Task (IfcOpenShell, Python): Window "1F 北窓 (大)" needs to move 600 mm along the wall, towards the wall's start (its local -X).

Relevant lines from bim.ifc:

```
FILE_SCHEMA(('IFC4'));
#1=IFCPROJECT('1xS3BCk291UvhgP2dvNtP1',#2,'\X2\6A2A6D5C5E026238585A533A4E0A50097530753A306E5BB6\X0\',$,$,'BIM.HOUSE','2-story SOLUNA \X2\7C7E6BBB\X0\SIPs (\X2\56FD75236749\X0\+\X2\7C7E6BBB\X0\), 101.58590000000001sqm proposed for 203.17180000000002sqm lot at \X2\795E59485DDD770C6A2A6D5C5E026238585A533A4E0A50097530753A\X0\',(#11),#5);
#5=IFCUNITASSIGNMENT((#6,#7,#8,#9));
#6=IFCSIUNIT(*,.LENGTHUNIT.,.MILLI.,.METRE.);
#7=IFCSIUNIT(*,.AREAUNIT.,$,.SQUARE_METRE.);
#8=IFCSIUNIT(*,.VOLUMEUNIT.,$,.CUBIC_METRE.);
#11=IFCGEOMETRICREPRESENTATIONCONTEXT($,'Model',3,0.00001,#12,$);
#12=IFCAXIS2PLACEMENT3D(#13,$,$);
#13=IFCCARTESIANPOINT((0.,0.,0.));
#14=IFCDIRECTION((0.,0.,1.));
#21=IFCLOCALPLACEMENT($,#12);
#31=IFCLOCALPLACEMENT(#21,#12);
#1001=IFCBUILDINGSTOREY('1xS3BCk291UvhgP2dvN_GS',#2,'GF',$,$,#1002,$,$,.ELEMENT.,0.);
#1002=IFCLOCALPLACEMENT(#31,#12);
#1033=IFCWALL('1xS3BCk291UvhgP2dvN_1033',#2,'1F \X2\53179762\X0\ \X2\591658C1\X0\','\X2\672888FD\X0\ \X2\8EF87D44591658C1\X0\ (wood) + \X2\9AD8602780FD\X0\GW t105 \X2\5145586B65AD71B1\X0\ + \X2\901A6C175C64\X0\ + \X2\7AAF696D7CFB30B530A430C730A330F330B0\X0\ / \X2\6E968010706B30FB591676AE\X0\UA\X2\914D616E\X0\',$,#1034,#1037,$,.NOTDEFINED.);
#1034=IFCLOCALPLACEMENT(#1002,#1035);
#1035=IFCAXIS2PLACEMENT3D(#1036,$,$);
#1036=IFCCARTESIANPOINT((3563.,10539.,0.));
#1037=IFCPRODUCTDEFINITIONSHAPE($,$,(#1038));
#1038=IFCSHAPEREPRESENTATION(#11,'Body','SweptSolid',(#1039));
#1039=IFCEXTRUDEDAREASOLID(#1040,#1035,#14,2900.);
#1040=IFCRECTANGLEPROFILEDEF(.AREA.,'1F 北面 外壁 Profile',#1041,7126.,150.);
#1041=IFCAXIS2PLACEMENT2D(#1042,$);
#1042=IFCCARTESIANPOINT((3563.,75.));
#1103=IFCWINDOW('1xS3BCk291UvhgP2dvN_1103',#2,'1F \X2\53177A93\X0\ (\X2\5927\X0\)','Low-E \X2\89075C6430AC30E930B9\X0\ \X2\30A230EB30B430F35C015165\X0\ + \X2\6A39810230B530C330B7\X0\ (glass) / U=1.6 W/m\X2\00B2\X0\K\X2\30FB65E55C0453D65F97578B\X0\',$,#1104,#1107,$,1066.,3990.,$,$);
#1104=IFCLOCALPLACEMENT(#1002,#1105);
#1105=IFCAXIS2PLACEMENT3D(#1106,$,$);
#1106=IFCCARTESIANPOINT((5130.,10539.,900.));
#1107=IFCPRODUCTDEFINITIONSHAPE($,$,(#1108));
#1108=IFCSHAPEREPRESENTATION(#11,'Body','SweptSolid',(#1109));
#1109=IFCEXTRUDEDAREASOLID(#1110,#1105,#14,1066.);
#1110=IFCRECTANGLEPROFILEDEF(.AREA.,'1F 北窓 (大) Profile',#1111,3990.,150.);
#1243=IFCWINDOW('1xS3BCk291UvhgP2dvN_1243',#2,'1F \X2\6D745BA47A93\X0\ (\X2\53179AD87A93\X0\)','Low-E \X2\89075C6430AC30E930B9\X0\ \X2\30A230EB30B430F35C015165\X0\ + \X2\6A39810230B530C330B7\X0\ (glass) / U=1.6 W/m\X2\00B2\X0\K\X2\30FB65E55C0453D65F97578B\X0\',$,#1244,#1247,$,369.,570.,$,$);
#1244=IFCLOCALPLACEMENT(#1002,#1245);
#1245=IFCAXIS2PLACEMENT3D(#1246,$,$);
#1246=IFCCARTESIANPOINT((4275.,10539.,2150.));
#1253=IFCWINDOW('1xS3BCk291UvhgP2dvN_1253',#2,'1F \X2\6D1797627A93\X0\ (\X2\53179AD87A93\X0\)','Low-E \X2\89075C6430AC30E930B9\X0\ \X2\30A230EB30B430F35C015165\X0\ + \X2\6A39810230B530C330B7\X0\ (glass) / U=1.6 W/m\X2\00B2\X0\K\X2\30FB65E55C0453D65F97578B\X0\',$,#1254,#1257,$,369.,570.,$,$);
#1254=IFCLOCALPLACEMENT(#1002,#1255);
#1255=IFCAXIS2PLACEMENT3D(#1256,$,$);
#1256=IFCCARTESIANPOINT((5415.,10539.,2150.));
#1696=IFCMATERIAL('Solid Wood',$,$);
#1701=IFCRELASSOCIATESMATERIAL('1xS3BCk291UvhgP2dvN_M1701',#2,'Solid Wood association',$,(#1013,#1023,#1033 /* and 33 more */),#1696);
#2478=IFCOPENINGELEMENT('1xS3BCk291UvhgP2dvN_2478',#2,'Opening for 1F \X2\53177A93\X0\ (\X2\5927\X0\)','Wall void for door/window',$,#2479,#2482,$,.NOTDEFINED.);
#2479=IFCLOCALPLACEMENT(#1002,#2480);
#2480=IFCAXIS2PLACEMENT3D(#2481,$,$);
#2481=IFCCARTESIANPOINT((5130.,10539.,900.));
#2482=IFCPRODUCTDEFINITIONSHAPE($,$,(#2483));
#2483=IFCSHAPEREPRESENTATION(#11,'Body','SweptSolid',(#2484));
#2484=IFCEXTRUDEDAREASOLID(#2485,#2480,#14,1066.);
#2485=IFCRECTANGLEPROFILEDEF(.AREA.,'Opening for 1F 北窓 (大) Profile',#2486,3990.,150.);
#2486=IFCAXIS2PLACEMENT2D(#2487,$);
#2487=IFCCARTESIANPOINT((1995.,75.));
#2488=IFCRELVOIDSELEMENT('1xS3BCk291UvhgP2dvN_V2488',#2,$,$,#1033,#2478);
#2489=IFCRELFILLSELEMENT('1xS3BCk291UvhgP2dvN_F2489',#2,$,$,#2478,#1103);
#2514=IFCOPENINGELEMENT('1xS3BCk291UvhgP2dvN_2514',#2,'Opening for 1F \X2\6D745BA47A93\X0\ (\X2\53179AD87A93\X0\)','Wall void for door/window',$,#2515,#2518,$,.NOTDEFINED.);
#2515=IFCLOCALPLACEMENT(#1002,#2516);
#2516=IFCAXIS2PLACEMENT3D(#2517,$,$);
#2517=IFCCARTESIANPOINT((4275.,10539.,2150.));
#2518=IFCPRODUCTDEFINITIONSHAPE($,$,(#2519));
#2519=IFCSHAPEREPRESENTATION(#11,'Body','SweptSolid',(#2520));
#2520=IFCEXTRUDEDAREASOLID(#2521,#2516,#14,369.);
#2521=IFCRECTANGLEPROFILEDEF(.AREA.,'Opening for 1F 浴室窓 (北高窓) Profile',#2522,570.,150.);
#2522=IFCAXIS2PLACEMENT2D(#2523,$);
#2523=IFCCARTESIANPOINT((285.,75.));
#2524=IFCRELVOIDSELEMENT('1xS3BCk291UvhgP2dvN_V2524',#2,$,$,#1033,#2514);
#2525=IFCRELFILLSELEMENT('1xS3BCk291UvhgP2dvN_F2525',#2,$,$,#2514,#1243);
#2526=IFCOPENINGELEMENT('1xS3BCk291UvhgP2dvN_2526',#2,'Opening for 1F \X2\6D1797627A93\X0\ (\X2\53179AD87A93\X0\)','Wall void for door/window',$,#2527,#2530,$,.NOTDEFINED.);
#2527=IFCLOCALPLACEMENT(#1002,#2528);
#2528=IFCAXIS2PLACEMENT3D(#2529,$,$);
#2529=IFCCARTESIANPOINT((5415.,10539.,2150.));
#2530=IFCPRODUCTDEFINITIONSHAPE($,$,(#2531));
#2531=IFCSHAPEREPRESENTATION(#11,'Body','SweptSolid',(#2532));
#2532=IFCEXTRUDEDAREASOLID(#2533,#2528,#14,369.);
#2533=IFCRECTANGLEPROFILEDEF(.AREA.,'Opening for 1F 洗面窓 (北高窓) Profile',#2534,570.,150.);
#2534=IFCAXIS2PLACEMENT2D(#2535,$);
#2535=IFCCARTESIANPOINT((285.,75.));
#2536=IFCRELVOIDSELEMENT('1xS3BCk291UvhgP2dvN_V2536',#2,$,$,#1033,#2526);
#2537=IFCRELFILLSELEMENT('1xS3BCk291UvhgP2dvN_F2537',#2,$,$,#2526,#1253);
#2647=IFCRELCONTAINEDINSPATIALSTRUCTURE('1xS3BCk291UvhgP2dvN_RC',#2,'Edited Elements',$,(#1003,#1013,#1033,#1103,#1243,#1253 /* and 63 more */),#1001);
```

```python
import ifcopenshell
import ifcopenshell.api.geometry
import ifcopenshell.util.placement
import ifcopenshell.util.unit

model = ifcopenshell.open("bim.ifc")
unit_scale = ifcopenshell.util.unit.calculate_unit_scale(model)

window = model.by_guid("1xS3BCk291UvhgP2dvN_1103")
opening = window.FillsVoids[0].RelatingOpeningElement
wall = opening.VoidsElements[0].RelatingBuildingElement

wall_matrix = ifcopenshell.util.placement.get_local_placement(wall.ObjectPlacement)
shift = wall_matrix[:3, 0] * -0.6 / unit_scale
before = ifcopenshell.util.placement.get_local_placement(window.ObjectPlacement)[:3, 3].copy()

# The window is not placed relative to its opening, so move both.
for product in (opening, window):
    matrix = ifcopenshell.util.placement.get_local_placement(product.ObjectPlacement)
    matrix[:3, 3] += shift
    ifcopenshell.api.geometry.edit_object_placement(model, product=product, matrix=matrix, is_si=False)

after = ifcopenshell.util.placement.get_local_placement(window.ObjectPlacement)[:3, 3]
print("window moved by", (after - before).round(3) + 0.0)

model.write("bim_rev.ifc")
```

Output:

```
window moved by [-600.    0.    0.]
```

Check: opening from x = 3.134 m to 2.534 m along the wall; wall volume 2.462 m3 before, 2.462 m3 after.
